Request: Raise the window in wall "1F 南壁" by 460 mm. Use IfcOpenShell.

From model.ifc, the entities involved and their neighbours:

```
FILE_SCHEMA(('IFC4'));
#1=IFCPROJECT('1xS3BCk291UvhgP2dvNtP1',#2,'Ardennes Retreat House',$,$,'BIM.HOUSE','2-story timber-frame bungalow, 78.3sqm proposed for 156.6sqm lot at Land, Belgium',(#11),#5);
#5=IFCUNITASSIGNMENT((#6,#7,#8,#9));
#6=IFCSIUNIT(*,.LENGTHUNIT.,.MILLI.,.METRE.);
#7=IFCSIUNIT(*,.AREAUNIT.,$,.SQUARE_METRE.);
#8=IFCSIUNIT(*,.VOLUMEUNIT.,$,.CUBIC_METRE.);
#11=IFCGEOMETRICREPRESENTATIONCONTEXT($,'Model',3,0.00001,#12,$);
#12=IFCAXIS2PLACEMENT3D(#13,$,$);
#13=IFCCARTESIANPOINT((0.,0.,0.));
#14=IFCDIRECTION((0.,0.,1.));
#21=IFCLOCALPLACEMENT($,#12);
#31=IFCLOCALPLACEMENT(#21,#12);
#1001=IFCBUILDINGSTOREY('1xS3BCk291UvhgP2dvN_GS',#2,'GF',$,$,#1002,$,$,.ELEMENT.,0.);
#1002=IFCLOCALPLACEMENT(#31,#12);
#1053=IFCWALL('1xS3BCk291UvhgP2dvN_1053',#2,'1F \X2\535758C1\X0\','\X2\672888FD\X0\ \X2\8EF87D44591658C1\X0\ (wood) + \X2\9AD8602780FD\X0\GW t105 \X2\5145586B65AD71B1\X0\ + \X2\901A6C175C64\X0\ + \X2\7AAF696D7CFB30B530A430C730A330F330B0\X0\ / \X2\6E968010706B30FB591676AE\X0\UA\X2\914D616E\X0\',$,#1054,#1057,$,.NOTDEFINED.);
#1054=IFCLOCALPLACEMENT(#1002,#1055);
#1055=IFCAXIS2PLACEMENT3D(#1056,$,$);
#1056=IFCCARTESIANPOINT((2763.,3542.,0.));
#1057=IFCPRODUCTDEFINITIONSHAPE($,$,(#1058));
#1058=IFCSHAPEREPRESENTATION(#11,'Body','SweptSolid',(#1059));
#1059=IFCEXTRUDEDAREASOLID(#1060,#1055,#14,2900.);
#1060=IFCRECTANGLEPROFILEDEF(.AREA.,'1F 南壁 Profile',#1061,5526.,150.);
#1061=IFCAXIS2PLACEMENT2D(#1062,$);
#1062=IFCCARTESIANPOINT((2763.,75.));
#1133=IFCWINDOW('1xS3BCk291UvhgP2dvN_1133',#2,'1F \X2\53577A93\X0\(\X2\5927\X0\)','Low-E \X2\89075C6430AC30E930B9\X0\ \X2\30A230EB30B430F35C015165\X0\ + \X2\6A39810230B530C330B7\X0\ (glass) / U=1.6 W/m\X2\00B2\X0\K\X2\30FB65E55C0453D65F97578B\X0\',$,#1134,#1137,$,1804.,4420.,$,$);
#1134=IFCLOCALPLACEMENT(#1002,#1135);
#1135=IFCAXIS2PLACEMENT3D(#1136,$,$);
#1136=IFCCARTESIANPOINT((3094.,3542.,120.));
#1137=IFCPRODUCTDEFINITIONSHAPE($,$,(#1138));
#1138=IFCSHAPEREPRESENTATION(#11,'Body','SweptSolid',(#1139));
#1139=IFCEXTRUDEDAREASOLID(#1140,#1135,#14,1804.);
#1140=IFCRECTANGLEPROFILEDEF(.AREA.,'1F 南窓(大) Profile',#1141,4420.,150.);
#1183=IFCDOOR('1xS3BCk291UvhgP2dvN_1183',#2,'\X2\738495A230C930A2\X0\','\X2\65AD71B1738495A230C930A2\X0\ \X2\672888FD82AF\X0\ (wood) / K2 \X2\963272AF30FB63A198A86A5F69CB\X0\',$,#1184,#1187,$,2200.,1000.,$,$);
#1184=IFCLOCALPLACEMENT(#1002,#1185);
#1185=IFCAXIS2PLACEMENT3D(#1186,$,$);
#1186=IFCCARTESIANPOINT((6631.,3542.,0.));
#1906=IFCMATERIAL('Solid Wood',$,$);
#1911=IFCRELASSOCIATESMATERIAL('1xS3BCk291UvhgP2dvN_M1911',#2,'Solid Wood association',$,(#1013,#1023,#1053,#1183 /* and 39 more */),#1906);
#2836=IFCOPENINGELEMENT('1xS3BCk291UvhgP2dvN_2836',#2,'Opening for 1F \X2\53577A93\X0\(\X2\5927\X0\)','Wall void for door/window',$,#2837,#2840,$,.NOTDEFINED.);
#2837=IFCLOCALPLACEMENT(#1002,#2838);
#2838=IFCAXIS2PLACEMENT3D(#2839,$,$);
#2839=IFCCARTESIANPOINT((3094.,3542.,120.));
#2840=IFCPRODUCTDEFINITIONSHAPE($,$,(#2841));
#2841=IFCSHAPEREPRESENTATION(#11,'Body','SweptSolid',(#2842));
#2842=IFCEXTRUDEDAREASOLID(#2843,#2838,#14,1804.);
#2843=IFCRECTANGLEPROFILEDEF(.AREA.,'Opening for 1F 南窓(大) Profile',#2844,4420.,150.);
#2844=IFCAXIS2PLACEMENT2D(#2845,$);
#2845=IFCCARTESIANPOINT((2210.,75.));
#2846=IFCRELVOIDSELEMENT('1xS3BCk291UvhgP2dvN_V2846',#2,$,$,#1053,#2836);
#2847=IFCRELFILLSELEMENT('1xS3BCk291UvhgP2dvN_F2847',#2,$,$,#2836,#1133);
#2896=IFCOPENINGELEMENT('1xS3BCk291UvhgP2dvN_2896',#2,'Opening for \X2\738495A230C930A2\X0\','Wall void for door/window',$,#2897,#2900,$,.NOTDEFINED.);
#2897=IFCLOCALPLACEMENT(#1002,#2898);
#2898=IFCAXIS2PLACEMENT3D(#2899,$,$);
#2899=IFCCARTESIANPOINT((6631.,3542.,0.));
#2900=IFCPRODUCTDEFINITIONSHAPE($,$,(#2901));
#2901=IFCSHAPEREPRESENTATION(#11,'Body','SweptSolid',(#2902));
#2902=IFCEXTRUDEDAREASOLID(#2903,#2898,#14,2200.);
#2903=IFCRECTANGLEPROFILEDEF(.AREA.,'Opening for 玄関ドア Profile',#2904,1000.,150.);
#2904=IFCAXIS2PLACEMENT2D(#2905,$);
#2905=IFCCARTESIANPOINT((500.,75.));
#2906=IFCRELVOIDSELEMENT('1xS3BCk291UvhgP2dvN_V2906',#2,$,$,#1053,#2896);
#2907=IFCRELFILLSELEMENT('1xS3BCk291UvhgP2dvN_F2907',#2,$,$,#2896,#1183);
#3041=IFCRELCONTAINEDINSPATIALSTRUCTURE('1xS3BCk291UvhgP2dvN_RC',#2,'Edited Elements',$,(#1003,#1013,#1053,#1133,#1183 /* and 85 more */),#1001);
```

```python
import numpy as np
import ifcopenshell
import ifcopenshell.api.geometry
import ifcopenshell.util.placement
import ifcopenshell.util.unit

model = ifcopenshell.open("model.ifc")
unit_scale = ifcopenshell.util.unit.calculate_unit_scale(model)

window = model.by_id(1133)
opening = window.FillsVoids[0].RelatingOpeningElement
dz = 0.46 / unit_scale

shift = np.array([0.0, 0.0, dz])
# The window is not placed relative to its opening, so move both.
for product in (opening, window):
    matrix = ifcopenshell.util.placement.get_local_placement(product.ObjectPlacement)
    matrix[:3, 3] += shift
    ifcopenshell.api.geometry.edit_object_placement(model, product=product, matrix=matrix, is_si=False)

print(f"moved by {dz * unit_scale:+.3f} m")

model.write("model-out.ifc")
```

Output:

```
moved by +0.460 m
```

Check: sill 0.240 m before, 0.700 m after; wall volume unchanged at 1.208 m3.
